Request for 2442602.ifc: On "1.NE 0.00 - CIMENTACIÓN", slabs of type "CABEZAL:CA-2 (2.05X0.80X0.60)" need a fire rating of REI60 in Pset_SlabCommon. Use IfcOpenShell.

First a look at what the model holds.

```python
import ifcopenshell
import ifcopenshell.util.element

model = ifcopenshell.open("2442602.ifc")
print(model.schema)
storey = next(s for s in model.by_type("IfcBuildingStorey") if s.Name == "1.NE 0.00 - CIMENTACIÓN")
slabs = [e for e in ifcopenshell.util.element.get_decomposition(storey) if e.is_a("IfcSlab")]
seen = {}
for e in slabs:
    element_type = ifcopenshell.util.element.get_type(e)
    key = (element_type.Name if element_type != e and element_type else None, ifcopenshell.util.element.get_pset(e, "Pset_SlabCommon", "FireRating"))
    seen[key] = seen.get(key, 0) + 1
for (name, value), count in sorted(seen.items(), key=str):
    print(count, "x", name, "|", value)
```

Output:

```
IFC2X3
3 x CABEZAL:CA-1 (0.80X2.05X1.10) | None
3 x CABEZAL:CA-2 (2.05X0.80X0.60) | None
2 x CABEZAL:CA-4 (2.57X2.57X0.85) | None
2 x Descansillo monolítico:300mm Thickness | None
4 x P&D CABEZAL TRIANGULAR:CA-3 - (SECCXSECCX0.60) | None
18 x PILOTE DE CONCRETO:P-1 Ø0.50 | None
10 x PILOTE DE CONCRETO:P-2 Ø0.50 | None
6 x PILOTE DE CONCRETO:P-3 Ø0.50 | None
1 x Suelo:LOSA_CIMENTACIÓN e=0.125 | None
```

```python
import ifcopenshell
import ifcopenshell.api.pset
import ifcopenshell.util.element

model = ifcopenshell.open("2442602.ifc")

storey = next(s for s in model.by_type("IfcBuildingStorey") if s.Name == "1.NE 0.00 - CIMENTACIÓN")
slabs = [e for e in ifcopenshell.util.element.get_decomposition(storey) if e.is_a("IfcSlab")]

count = 0
for e in slabs:
    element_type = ifcopenshell.util.element.get_type(e)
    if element_type in (None, e) or element_type.Name != "CABEZAL:CA-2 (2.05X0.80X0.60)":
        continue
    # add_pset returns the element's existing set when there is one.
    pset = ifcopenshell.api.pset.add_pset(model, product=e, name="Pset_SlabCommon")
    ifcopenshell.api.pset.edit_pset(model, pset=pset, properties={"FireRating": "REI60"})
    count += 1

print(count, "slabs updated")

model.write("2442602_rev.ifc")
```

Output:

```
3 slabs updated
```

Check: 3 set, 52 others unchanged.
